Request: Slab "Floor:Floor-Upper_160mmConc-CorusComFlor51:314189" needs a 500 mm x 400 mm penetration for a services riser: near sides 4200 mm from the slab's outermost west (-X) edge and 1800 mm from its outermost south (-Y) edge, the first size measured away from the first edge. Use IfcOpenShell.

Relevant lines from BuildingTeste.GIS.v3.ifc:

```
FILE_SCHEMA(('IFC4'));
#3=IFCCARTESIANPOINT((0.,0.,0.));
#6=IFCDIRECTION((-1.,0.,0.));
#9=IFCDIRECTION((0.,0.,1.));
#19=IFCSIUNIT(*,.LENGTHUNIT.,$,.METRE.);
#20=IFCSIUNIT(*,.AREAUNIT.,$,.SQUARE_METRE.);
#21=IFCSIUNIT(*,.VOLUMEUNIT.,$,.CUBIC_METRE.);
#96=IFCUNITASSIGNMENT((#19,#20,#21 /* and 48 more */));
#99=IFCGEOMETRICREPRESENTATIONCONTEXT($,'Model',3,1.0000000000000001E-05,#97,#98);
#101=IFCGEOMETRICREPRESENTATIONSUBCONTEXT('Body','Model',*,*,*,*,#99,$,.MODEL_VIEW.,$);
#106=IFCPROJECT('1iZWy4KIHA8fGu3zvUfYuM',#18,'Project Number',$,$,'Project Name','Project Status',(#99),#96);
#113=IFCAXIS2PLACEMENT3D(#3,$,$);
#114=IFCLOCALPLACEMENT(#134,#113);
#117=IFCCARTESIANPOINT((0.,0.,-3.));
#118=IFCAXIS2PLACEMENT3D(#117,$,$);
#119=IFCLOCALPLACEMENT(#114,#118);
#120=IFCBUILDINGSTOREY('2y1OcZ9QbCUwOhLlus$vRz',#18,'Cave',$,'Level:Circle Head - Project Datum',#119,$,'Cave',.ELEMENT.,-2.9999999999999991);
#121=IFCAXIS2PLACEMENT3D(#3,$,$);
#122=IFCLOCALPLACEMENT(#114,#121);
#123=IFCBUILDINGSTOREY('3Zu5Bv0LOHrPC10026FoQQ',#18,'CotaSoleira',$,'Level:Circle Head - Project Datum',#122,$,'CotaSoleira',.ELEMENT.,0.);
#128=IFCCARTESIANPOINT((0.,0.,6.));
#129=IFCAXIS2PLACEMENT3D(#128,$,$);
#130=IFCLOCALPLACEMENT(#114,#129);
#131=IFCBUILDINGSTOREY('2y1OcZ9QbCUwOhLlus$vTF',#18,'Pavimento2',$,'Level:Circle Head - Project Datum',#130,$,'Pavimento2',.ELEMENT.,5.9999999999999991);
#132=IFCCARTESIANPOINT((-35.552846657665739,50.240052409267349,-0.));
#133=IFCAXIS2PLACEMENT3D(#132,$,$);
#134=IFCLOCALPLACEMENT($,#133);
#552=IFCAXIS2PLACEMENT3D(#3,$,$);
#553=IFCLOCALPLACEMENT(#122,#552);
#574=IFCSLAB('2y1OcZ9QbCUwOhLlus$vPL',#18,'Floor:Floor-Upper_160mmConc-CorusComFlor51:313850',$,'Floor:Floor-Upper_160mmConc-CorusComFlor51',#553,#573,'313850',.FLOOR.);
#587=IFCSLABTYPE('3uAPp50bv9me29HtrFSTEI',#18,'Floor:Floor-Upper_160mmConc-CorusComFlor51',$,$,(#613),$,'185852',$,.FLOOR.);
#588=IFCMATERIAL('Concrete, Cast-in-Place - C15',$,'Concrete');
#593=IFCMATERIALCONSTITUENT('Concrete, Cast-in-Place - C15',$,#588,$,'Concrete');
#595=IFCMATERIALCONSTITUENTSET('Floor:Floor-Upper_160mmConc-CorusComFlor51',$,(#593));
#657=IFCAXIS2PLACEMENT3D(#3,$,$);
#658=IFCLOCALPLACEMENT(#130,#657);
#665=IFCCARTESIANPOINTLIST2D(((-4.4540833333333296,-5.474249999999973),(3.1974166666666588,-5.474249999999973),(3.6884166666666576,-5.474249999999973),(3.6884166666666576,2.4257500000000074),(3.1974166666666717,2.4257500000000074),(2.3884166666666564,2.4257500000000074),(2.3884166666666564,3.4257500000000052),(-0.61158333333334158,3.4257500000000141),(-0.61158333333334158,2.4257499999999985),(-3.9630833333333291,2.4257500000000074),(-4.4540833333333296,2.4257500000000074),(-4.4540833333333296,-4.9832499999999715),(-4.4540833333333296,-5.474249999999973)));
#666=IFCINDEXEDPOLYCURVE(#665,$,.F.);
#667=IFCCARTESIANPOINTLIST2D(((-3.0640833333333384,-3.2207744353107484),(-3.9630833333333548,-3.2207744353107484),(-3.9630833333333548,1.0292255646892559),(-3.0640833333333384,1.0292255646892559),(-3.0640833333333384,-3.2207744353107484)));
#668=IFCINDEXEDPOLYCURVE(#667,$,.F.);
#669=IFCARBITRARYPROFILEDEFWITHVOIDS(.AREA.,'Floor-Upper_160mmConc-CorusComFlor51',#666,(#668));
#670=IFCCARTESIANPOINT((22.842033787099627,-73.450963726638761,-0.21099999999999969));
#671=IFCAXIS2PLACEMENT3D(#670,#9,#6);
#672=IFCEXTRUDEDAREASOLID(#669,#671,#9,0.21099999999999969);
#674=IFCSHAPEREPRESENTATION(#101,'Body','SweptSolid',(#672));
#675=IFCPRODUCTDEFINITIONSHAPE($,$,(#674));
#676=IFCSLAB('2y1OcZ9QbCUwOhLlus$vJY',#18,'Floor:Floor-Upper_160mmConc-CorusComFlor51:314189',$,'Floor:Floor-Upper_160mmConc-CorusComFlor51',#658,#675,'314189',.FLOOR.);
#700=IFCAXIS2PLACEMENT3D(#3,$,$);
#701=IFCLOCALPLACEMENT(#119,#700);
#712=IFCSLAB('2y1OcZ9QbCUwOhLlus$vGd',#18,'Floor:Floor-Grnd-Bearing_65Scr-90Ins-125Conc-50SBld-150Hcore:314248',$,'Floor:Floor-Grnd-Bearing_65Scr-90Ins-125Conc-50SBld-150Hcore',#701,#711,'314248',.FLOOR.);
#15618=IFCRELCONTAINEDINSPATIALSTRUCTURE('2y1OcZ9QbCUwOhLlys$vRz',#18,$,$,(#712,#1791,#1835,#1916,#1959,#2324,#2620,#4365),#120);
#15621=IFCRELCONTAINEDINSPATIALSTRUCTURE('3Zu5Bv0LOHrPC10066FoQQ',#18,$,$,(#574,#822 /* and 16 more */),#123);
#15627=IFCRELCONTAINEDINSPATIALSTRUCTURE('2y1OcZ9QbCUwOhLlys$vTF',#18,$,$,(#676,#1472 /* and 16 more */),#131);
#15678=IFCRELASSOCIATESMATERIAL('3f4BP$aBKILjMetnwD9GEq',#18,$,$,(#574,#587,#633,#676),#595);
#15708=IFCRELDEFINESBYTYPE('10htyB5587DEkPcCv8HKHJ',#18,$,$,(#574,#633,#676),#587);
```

```python
import numpy as np
import ifcopenshell
import ifcopenshell.api.feature
import ifcopenshell.api.geometry
import ifcopenshell.api.root
import ifcopenshell.geom
import ifcopenshell.util.placement
import ifcopenshell.util.representation
import ifcopenshell.util.shape
import ifcopenshell.util.unit

model = ifcopenshell.open("BuildingTeste.GIS.v3.ifc")
unit_scale = ifcopenshell.util.unit.calculate_unit_scale(model)
settings = ifcopenshell.geom.settings()


def volume(element):
    """Net volume in cubic metres, openings subtracted."""
    shape = ifcopenshell.geom.create_shape(settings, element)
    return ifcopenshell.util.shape.get_volume(shape.geometry)


slab = model.by_guid("2y1OcZ9QbCUwOhLlus$vJY")
before = volume(slab)

# Extent in the slab's own axes, in metres. The edges named are its -X and -Y sides.
slab_shape = ifcopenshell.geom.create_shape(settings, slab)
vertices = ifcopenshell.util.shape.get_vertices(slab_shape.geometry)
x_min, y_min, bottom = vertices.min(axis=0)
top = vertices[:, 2].max()

opening = ifcopenshell.api.root.create_entity(model, ifc_class="IfcOpeningElement", name="Services riser opening", predefined_type="OPENING")
context = ifcopenshell.util.representation.get_context(model, "Model", "Body", "MODEL_VIEW")
width, depth = 0.5, 0.4
outline = [(0.0, 0.0), (width, 0.0), (width, depth), (0.0, depth), (0.0, 0.0)]
# Overshoot both faces by 50 mm so the cut is clean.
shape = ifcopenshell.api.geometry.add_slab_representation(
    model, context=context, depth=top - bottom + 0.1, polyline=outline
)
ifcopenshell.api.geometry.assign_representation(model, product=opening, representation=shape)

matrix = ifcopenshell.util.placement.get_local_placement(slab.ObjectPlacement)
matrix[:, 3] = matrix @ np.append(np.array([x_min + 4.2, y_min + 1.8, bottom - 0.05]) / unit_scale, 1.0)
ifcopenshell.api.geometry.edit_object_placement(model, product=opening, matrix=matrix, is_si=False)
ifcopenshell.api.feature.add_feature(model, feature=opening, element=slab)

after = volume(slab)

print(f"slab volume {before:.3f} -> {after:.3f} m3")

model.write("BuildingTeste.GIS.v3_edited.ifc")
```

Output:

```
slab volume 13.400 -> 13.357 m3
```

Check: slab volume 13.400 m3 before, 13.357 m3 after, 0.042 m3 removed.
